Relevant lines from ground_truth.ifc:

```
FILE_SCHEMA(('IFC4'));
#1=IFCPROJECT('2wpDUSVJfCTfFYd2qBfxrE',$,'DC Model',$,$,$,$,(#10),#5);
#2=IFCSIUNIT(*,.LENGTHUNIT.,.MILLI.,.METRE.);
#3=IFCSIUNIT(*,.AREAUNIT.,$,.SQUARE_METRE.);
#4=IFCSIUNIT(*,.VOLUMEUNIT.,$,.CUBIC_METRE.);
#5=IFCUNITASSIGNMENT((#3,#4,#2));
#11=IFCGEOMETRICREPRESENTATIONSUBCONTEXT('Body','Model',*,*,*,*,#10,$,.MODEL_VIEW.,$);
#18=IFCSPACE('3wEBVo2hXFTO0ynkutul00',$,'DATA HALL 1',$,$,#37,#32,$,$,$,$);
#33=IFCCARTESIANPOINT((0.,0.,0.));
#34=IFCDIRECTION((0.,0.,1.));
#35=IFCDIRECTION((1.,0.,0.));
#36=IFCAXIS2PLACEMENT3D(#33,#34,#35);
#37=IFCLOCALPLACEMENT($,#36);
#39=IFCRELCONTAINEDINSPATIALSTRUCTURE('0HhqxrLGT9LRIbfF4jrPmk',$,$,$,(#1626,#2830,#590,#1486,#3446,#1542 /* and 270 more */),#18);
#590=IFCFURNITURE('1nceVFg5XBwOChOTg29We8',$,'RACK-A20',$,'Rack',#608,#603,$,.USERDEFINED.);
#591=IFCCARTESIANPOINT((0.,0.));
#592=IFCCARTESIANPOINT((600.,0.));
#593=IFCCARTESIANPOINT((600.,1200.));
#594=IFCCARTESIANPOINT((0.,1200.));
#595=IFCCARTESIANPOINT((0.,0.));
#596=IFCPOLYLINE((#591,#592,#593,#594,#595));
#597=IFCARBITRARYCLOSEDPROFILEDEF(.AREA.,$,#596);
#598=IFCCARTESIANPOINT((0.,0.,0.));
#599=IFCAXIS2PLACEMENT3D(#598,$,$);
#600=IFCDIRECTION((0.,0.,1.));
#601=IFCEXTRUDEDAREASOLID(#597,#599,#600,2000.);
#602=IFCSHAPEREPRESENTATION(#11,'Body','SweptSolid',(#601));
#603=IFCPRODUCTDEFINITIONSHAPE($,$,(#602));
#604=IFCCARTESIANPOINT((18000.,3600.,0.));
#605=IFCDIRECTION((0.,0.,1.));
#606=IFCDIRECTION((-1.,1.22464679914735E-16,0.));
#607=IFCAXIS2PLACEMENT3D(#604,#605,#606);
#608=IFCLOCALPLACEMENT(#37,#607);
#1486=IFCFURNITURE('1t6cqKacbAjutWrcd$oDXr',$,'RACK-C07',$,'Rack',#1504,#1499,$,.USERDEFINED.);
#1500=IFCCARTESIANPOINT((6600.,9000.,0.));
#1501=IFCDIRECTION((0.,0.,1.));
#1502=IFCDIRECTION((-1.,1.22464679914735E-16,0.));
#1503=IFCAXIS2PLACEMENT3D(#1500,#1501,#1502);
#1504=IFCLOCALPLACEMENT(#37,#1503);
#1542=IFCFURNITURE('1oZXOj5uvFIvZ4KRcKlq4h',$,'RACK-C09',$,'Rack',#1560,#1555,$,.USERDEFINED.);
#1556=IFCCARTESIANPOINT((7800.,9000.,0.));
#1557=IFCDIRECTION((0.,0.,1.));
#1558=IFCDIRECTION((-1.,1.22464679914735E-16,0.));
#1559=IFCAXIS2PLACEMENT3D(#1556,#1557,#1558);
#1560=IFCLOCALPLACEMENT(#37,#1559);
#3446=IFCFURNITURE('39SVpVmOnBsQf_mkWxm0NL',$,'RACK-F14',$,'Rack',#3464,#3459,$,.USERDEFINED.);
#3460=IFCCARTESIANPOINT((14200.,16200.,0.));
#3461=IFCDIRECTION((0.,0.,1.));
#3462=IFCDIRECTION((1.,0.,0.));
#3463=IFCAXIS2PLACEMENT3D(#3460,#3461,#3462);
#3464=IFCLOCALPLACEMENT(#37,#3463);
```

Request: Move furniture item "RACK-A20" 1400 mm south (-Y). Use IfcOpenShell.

```python
import ifcopenshell
import ifcopenshell.api.geometry
import ifcopenshell.util.placement

model = ifcopenshell.open("ground_truth.ifc")

item = model.by_guid("1nceVFg5XBwOChOTg29We8")
matrix = ifcopenshell.util.placement.get_local_placement(item.ObjectPlacement)
matrix[1, 3] -= 1400.0
ifcopenshell.api.geometry.edit_object_placement(model, product=item, matrix=matrix, is_si=False)

print(ifcopenshell.util.placement.get_local_placement(item.ObjectPlacement).round(3) + 0.0)

model.write("ground_truth-out.ifc")
```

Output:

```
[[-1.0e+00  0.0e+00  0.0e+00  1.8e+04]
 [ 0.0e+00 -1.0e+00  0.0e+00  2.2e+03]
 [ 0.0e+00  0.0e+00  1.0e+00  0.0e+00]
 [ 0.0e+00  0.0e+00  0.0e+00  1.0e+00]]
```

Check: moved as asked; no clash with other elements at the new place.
